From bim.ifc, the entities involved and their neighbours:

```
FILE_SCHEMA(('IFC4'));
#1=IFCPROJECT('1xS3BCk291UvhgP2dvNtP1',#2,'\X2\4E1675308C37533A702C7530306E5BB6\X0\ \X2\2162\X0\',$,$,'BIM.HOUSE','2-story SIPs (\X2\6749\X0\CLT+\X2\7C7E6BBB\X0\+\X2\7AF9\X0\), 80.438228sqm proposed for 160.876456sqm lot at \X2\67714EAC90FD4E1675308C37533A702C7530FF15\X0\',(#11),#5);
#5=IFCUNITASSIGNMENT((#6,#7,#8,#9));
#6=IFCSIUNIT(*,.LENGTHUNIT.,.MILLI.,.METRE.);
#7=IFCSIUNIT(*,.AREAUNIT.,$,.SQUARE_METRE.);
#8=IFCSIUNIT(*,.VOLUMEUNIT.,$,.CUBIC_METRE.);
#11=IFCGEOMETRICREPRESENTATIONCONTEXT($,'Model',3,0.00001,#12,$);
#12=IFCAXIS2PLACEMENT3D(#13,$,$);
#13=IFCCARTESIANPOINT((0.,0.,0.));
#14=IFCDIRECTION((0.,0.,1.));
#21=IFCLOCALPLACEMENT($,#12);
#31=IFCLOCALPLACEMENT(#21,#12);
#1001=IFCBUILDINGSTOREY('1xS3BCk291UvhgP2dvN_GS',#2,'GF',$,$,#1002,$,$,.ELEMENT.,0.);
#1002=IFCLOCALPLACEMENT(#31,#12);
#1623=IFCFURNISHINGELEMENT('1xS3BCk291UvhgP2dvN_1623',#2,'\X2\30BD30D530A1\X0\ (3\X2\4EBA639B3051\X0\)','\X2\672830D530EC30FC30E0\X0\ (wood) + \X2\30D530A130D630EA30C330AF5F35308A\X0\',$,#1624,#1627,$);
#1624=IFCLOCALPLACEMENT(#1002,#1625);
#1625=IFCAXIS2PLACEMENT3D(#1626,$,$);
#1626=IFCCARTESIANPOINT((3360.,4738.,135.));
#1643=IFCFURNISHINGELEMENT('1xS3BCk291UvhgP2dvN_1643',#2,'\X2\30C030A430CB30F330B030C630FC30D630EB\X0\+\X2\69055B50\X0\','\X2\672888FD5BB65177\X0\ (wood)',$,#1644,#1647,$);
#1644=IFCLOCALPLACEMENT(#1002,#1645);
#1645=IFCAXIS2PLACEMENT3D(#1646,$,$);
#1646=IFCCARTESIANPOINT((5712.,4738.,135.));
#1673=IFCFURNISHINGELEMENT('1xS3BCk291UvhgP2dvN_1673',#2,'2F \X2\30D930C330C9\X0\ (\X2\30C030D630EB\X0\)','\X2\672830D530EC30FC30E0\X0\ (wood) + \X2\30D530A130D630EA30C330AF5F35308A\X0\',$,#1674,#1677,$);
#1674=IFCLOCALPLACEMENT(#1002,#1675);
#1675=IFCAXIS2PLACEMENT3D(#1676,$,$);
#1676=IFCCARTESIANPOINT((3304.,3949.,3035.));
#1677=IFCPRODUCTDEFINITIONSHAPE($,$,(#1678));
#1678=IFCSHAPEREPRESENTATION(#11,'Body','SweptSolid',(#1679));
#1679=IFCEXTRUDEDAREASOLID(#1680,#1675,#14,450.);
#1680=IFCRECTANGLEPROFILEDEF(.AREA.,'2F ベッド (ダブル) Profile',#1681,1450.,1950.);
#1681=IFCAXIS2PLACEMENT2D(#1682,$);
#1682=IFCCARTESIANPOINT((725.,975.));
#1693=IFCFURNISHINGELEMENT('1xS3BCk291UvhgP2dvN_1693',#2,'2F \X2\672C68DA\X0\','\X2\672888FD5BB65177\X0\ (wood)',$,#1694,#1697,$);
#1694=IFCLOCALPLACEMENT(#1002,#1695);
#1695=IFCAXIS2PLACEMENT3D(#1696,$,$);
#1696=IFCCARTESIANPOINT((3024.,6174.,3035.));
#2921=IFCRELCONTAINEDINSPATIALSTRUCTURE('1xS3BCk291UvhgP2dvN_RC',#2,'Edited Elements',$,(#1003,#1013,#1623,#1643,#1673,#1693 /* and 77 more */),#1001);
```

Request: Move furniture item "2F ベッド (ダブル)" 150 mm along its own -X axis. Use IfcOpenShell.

```python
import ifcopenshell
import ifcopenshell.api.geometry
import ifcopenshell.util.placement
import ifcopenshell.util.unit

model = ifcopenshell.open("bim.ifc")
unit_scale = ifcopenshell.util.unit.calculate_unit_scale(model)

item = model.by_guid("1xS3BCk291UvhgP2dvN_1673")
matrix = ifcopenshell.util.placement.get_local_placement(item.ObjectPlacement)
matrix[:3, 3] -= matrix[:3, 0] * 0.15 / unit_scale
ifcopenshell.api.geometry.edit_object_placement(model, product=item, matrix=matrix, is_si=False)

print(ifcopenshell.util.placement.get_local_placement(item.ObjectPlacement).round(3) + 0.0)

model.write("bim_edited.ifc")
```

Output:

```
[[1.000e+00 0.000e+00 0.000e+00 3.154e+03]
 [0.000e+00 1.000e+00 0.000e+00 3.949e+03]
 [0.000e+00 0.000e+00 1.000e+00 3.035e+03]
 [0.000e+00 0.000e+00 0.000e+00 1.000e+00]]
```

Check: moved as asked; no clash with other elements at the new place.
